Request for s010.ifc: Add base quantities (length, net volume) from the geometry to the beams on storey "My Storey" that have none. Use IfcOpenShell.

First a look at what the model holds.

```python
import ifcopenshell
import ifcopenshell.util.element
import ifcopenshell.util.unit

model = ifcopenshell.open("s010.ifc")
print(model.schema)
for unit_type in ("LENGTHUNIT", "AREAUNIT", "VOLUMEUNIT"):
    print(unit_type, ifcopenshell.util.unit.calculate_unit_scale(model, unit_type))
storey = next(s for s in model.by_type("IfcBuildingStorey") if s.Name == "My Storey")
beams = [e for e in ifcopenshell.util.element.get_decomposition(storey) if e.is_a("IfcBeam")]
for e in sorted(beams, key=lambda e: e.id()):
    print(e.id(), e.is_a(), e.Name, list(ifcopenshell.util.element.get_psets(e, qtos_only=True)), sep=" | ")
```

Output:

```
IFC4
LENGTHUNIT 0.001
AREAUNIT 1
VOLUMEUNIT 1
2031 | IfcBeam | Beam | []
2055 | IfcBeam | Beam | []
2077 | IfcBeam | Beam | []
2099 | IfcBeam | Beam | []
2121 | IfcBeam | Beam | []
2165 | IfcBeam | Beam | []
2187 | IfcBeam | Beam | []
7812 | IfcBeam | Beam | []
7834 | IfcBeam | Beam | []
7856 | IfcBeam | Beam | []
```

```python
import ifcopenshell
import ifcopenshell.api.pset
import ifcopenshell.geom
import ifcopenshell.util.element
import ifcopenshell.util.shape
import ifcopenshell.util.unit

model = ifcopenshell.open("s010.ifc")
unit_scale = ifcopenshell.util.unit.calculate_unit_scale(model)
volume_scale = ifcopenshell.util.unit.calculate_unit_scale(model, "VOLUMEUNIT")
settings = ifcopenshell.geom.settings()

storey = next(s for s in model.by_type("IfcBuildingStorey") if s.Name == "My Storey")
beams = [e for e in ifcopenshell.util.element.get_decomposition(storey) if e.is_a("IfcBeam")]

for e in sorted(beams, key=lambda e: e.id()):
    if ifcopenshell.util.element.get_psets(e, qtos_only=True, should_inherit=False):
        continue
    # Geometry comes back in metres, in the element's own axes.
    shape = ifcopenshell.geom.create_shape(settings, e)
    values = {
        "Length": ifcopenshell.util.shape.get_max_xyz(shape.geometry) / unit_scale,
        "NetVolume": ifcopenshell.util.shape.get_volume(shape.geometry) / volume_scale,
    }
    qto = ifcopenshell.api.pset.add_qto(model, product=e, name="Qto_BeamBaseQuantities")
    ifcopenshell.api.pset.edit_qto(model, qto=qto, properties=values)
    print(e.id(), {k: round(v, 3) for k, v in values.items()})

model.write("s010_rev.ifc")
```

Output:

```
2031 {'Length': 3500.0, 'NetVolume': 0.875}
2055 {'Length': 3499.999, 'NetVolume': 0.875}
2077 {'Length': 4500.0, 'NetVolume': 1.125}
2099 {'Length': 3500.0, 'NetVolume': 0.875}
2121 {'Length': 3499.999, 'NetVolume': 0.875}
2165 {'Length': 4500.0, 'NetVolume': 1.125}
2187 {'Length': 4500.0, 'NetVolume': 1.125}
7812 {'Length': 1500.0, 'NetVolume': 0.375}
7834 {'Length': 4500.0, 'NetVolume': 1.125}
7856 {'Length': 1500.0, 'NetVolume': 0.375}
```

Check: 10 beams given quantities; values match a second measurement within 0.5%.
